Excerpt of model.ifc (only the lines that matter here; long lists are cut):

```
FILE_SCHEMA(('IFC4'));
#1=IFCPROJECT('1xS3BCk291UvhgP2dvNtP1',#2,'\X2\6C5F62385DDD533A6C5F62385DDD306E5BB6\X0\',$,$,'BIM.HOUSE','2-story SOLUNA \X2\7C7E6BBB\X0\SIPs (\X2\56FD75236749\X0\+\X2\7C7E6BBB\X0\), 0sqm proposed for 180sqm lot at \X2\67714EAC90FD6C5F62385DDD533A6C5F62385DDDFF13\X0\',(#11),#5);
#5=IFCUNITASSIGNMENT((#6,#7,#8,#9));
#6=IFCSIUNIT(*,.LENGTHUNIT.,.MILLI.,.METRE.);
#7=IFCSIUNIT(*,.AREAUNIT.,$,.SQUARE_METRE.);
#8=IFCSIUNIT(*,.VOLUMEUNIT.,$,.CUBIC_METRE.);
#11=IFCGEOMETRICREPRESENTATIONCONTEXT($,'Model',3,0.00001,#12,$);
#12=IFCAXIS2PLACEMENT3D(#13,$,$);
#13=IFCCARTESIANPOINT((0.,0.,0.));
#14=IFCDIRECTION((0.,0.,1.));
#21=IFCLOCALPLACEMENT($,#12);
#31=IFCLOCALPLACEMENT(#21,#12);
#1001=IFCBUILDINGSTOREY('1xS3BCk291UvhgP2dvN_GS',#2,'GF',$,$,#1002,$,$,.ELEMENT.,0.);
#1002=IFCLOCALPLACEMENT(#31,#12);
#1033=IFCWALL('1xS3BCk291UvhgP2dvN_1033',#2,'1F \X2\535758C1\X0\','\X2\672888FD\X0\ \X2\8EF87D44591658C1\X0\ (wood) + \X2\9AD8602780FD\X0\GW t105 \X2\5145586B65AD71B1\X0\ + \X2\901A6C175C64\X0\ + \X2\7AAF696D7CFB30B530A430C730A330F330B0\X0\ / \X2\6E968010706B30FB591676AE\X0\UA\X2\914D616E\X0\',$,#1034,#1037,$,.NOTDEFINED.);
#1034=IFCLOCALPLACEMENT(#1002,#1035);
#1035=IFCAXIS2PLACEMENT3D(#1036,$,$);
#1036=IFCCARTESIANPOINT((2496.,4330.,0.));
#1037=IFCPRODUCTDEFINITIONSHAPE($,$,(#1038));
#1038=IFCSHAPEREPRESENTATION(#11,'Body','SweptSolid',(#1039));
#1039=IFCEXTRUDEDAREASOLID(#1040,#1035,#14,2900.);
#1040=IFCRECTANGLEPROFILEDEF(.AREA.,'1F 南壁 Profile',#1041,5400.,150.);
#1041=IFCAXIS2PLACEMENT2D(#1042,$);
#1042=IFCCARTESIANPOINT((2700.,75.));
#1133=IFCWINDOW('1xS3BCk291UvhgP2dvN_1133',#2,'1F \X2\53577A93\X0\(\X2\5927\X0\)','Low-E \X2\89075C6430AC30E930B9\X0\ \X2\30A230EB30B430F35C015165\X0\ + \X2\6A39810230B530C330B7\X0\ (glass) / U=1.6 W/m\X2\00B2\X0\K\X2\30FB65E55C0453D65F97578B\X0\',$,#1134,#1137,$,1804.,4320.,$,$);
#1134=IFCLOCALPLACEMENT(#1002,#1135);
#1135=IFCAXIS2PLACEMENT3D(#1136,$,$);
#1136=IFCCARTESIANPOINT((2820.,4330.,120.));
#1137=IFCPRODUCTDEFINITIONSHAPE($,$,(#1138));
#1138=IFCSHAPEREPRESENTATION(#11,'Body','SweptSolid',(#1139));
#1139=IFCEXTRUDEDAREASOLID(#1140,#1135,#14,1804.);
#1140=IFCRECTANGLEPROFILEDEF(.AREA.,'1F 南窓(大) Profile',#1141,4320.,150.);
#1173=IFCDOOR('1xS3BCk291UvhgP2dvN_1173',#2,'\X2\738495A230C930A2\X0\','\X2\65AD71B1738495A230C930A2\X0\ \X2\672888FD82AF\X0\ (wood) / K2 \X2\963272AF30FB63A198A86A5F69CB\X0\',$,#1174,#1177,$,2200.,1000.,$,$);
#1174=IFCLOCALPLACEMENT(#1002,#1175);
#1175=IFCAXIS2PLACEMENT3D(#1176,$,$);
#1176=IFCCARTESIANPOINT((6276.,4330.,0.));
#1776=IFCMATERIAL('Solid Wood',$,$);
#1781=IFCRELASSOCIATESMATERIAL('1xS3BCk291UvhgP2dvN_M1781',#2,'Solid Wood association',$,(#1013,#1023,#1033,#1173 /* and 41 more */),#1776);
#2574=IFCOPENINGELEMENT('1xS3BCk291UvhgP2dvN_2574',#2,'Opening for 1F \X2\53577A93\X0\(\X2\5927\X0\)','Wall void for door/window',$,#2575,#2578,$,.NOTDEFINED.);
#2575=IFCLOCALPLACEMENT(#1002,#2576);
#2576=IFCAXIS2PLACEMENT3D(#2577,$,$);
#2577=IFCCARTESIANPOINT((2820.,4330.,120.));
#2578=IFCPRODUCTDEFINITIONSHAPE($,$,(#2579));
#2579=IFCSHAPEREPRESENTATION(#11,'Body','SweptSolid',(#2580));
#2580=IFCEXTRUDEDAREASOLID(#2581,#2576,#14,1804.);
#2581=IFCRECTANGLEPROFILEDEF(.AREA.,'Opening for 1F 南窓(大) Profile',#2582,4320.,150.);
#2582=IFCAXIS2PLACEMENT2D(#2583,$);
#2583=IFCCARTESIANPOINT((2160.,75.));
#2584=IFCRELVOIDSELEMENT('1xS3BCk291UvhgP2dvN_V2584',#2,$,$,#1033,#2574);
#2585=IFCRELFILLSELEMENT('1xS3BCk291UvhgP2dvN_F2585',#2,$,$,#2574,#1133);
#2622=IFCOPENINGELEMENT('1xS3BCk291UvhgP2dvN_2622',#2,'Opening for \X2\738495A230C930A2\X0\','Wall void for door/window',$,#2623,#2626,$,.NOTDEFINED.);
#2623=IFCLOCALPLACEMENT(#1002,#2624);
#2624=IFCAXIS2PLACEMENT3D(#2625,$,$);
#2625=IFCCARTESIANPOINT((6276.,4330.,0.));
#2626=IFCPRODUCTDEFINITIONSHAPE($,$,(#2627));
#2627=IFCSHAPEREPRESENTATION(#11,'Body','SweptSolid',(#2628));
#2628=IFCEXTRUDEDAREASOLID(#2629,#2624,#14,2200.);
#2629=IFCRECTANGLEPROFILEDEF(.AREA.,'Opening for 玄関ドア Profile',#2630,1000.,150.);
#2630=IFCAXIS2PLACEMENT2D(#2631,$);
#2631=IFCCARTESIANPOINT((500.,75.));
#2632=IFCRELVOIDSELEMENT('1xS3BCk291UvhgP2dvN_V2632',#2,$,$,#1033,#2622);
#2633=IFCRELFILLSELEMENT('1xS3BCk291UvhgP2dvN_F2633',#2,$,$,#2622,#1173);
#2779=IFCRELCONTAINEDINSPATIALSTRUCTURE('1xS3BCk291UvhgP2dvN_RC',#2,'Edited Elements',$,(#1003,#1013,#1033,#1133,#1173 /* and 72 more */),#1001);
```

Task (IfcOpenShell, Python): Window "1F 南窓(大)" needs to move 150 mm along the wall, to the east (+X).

```python
import ifcopenshell
import ifcopenshell.api.geometry
import ifcopenshell.util.placement

model = ifcopenshell.open("model.ifc")

window = model.by_guid("1xS3BCk291UvhgP2dvN_1133")
opening = window.FillsVoids[0].RelatingOpeningElement
wall = opening.VoidsElements[0].RelatingBuildingElement

wall_matrix = ifcopenshell.util.placement.get_local_placement(wall.ObjectPlacement)
shift = wall_matrix[:3, 0] * 150.0
before = ifcopenshell.util.placement.get_local_placement(window.ObjectPlacement)[:3, 3].copy()

# The window is not placed relative to its opening, so move both.
for product in (opening, window):
    matrix = ifcopenshell.util.placement.get_local_placement(product.ObjectPlacement)
    matrix[:3, 3] += shift
    ifcopenshell.api.geometry.edit_object_placement(model, product=product, matrix=matrix, is_si=False)

after = ifcopenshell.util.placement.get_local_placement(window.ObjectPlacement)[:3, 3]
print("window moved by", (after - before).round(3) + 0.0)

model.write("model-out.ifc")
```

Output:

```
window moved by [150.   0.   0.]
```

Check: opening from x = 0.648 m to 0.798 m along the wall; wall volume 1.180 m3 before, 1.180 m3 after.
